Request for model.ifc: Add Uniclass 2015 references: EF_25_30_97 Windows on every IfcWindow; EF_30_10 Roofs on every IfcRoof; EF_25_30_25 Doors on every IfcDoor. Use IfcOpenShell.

First a look at what the model holds.

```python
import ifcopenshell

model = ifcopenshell.open("model.ifc")
print(model.schema)
print("classifications:", [c.Name for c in model.by_type("IfcClassification")])
for ifc_class in ("IfcDoor", "IfcRoof", "IfcStair", "IfcWall", "IfcWindow"):
    print(ifc_class, len(model.by_type(ifc_class)))
```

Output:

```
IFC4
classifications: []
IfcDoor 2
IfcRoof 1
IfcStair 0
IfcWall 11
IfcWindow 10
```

```python
import ifcopenshell
import ifcopenshell.api.classification

model = ifcopenshell.open("model.ifc")

system = ifcopenshell.api.classification.add_classification(model, classification="Uniclass 2015")

codes = {
    "IfcWindow": ("EF_25_30_97", "Windows"),
    "IfcRoof": ("EF_30_10", "Roofs"),
    "IfcDoor": ("EF_25_30_25", "Doors"),
}
for ifc_class, (code, name) in codes.items():
    products = model.by_type(ifc_class)
    ifcopenshell.api.classification.add_reference(
        model, products=products, classification=system, identification=code, name=name
    )
    print(code, len(products))

model.write("model_edited.ifc")
```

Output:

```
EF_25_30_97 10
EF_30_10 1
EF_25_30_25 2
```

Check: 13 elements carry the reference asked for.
